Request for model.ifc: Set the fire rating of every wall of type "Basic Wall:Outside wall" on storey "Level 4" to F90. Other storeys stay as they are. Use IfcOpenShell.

First a look at what the model holds.

```python
import ifcopenshell
import ifcopenshell.util.element

model = ifcopenshell.open("model.ifc")
print(model.schema)
storey = next(s for s in model.by_type("IfcBuildingStorey") if s.Name == "Level 4")
walls = [e for e in ifcopenshell.util.element.get_decomposition(storey) if e.is_a("IfcWall")]
seen = {}
for e in walls:
    element_type = ifcopenshell.util.element.get_type(e)
    key = (element_type.Name if element_type != e and element_type else None, ifcopenshell.util.element.get_pset(e, "Pset_WallCommon", "FireRating"))
    seen[key] = seen.get(key, 0) + 1
for (name, value), count in sorted(seen.items(), key=str):
    print(count, "x", name, "|", value)
```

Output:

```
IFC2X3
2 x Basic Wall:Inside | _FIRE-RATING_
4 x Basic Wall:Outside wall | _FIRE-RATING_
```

```python
import ifcopenshell
import ifcopenshell.api.pset
import ifcopenshell.util.element

model = ifcopenshell.open("model.ifc")

storey = next(s for s in model.by_type("IfcBuildingStorey") if s.Name == "Level 4")
walls = [e for e in ifcopenshell.util.element.get_decomposition(storey) if e.is_a("IfcWall")]

count = 0
for e in walls:
    element_type = ifcopenshell.util.element.get_type(e)
    if element_type in (None, e) or element_type.Name != "Basic Wall:Outside wall":
        continue
    # add_pset returns the element's existing set when there is one.
    pset = ifcopenshell.api.pset.add_pset(model, product=e, name="Pset_WallCommon")
    ifcopenshell.api.pset.edit_pset(model, pset=pset, properties={"FireRating": "F90"})
    count += 1

print(count, "walls updated")

model.write("model_v2.ifc")
```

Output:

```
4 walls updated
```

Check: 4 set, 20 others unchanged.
